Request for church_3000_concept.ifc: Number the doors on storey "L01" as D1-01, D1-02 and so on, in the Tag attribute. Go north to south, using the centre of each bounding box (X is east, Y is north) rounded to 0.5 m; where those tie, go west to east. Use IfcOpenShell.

First a look at what the model holds.

```python
import ifcopenshell
import ifcopenshell.util.element
import ifcopenshell.util.placement

model = ifcopenshell.open("church_3000_concept.ifc")
print(model.schema)
storey = next(s for s in model.by_type("IfcBuildingStorey") if s.Name == "L01")
doors = [e for e in ifcopenshell.util.element.get_decomposition(storey) if e.is_a("IfcDoor")]
for e in sorted(doors, key=lambda e: e.id()):
    origin = ifcopenshell.util.placement.get_local_placement(e.ObjectPlacement)[:3, 3]
    print(e.id(), e.Tag, e.Name, origin.round(2) + 0.0, sep=" | ")
```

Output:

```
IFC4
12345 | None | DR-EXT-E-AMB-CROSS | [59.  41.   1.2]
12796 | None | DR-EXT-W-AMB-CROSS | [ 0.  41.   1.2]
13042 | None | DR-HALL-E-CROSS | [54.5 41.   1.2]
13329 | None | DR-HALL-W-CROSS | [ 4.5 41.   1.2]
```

```python
import ifcopenshell
import ifcopenshell.geom
import ifcopenshell.util.element
import ifcopenshell.util.shape

model = ifcopenshell.open("church_3000_concept.ifc")
settings = ifcopenshell.geom.settings()
settings.set("use-world-coords", True)


def centre(element):
    shape = ifcopenshell.geom.create_shape(settings, element)
    return ifcopenshell.util.shape.get_bbox_centroid(shape.geometry)


storey = next(s for s in model.by_type("IfcBuildingStorey") if s.Name == "L01")
doors = [e for e in ifcopenshell.util.element.get_decomposition(storey) if e.is_a("IfcDoor")]

# Insertion points can sit at a corner or the storey origin, so sort by the geometry (in metres).
centres = {e: centre(e) for e in doors}
doors.sort(key=lambda e: (-round(centres[e][1] / 0.5), centres[e][0]))

for i, e in enumerate(doors, start=1):
    number = f"D1-{i:02d}"
    e.Tag = number
    print(e.id(), number)

model.write("church_3000_concept_rev.ifc")
```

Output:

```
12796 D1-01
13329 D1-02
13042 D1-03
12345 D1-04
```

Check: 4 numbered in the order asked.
